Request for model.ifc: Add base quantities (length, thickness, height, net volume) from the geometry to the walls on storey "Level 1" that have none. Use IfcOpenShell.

First a look at what the model holds.

```python
import ifcopenshell
import ifcopenshell.util.element
import ifcopenshell.util.unit

model = ifcopenshell.open("model.ifc")
print(model.schema)
for unit_type in ("LENGTHUNIT", "AREAUNIT", "VOLUMEUNIT"):
    print(unit_type, ifcopenshell.util.unit.calculate_unit_scale(model, unit_type))
storey = next(s for s in model.by_type("IfcBuildingStorey") if s.Name == "Level 1")
walls = [e for e in ifcopenshell.util.element.get_decomposition(storey) if e.is_a("IfcWall")]
for e in sorted(walls, key=lambda e: e.id()):
    print(e.id(), e.is_a(), e.Name, list(ifcopenshell.util.element.get_psets(e, qtos_only=True)), sep=" | ")
```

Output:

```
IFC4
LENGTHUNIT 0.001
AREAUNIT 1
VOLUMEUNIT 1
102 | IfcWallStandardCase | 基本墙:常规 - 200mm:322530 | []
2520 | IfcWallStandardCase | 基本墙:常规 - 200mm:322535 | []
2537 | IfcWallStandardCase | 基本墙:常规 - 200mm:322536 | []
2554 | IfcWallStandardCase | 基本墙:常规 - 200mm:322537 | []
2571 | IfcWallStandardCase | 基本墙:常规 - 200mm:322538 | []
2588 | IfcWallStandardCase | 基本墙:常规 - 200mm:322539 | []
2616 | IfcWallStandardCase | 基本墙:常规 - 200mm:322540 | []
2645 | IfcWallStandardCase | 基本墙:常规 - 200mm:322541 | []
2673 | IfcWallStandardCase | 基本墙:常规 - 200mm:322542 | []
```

```python
import ifcopenshell
import ifcopenshell.api.pset
import ifcopenshell.geom
import ifcopenshell.util.element
import ifcopenshell.util.shape
import ifcopenshell.util.unit

model = ifcopenshell.open("model.ifc")
unit_scale = ifcopenshell.util.unit.calculate_unit_scale(model)
volume_scale = ifcopenshell.util.unit.calculate_unit_scale(model, "VOLUMEUNIT")
settings = ifcopenshell.geom.settings()

storey = next(s for s in model.by_type("IfcBuildingStorey") if s.Name == "Level 1")
walls = [e for e in ifcopenshell.util.element.get_decomposition(storey) if e.is_a("IfcWall")]

for e in sorted(walls, key=lambda e: e.id()):
    if ifcopenshell.util.element.get_psets(e, qtos_only=True, should_inherit=False):
        continue
    # Geometry comes back in metres, in the element's own axes.
    shape = ifcopenshell.geom.create_shape(settings, e)
    values = {
        "Length": ifcopenshell.util.shape.get_x(shape.geometry) / unit_scale,
        "Width": ifcopenshell.util.shape.get_y(shape.geometry) / unit_scale,
        "Height": ifcopenshell.util.shape.get_z(shape.geometry) / unit_scale,
        "NetVolume": ifcopenshell.util.shape.get_volume(shape.geometry) / volume_scale,
    }
    qto = ifcopenshell.api.pset.add_qto(model, product=e, name="Qto_WallBaseQuantities")
    ifcopenshell.api.pset.edit_qto(model, qto=qto, properties=values)
    print(e.id(), {k: round(v, 3) for k, v in values.items()})

model.write("model_edited.ifc")
```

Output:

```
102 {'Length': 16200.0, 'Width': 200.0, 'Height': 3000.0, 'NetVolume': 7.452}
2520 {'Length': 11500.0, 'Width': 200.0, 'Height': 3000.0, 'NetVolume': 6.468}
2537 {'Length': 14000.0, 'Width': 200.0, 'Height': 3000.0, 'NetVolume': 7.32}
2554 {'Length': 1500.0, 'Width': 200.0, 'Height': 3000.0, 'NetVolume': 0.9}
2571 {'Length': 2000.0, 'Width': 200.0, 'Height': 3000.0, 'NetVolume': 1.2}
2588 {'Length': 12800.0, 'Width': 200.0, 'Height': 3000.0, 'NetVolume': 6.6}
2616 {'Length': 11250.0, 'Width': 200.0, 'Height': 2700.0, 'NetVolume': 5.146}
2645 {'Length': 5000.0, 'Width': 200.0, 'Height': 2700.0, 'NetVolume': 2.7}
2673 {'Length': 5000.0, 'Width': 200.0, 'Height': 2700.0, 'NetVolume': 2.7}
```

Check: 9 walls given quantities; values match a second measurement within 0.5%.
